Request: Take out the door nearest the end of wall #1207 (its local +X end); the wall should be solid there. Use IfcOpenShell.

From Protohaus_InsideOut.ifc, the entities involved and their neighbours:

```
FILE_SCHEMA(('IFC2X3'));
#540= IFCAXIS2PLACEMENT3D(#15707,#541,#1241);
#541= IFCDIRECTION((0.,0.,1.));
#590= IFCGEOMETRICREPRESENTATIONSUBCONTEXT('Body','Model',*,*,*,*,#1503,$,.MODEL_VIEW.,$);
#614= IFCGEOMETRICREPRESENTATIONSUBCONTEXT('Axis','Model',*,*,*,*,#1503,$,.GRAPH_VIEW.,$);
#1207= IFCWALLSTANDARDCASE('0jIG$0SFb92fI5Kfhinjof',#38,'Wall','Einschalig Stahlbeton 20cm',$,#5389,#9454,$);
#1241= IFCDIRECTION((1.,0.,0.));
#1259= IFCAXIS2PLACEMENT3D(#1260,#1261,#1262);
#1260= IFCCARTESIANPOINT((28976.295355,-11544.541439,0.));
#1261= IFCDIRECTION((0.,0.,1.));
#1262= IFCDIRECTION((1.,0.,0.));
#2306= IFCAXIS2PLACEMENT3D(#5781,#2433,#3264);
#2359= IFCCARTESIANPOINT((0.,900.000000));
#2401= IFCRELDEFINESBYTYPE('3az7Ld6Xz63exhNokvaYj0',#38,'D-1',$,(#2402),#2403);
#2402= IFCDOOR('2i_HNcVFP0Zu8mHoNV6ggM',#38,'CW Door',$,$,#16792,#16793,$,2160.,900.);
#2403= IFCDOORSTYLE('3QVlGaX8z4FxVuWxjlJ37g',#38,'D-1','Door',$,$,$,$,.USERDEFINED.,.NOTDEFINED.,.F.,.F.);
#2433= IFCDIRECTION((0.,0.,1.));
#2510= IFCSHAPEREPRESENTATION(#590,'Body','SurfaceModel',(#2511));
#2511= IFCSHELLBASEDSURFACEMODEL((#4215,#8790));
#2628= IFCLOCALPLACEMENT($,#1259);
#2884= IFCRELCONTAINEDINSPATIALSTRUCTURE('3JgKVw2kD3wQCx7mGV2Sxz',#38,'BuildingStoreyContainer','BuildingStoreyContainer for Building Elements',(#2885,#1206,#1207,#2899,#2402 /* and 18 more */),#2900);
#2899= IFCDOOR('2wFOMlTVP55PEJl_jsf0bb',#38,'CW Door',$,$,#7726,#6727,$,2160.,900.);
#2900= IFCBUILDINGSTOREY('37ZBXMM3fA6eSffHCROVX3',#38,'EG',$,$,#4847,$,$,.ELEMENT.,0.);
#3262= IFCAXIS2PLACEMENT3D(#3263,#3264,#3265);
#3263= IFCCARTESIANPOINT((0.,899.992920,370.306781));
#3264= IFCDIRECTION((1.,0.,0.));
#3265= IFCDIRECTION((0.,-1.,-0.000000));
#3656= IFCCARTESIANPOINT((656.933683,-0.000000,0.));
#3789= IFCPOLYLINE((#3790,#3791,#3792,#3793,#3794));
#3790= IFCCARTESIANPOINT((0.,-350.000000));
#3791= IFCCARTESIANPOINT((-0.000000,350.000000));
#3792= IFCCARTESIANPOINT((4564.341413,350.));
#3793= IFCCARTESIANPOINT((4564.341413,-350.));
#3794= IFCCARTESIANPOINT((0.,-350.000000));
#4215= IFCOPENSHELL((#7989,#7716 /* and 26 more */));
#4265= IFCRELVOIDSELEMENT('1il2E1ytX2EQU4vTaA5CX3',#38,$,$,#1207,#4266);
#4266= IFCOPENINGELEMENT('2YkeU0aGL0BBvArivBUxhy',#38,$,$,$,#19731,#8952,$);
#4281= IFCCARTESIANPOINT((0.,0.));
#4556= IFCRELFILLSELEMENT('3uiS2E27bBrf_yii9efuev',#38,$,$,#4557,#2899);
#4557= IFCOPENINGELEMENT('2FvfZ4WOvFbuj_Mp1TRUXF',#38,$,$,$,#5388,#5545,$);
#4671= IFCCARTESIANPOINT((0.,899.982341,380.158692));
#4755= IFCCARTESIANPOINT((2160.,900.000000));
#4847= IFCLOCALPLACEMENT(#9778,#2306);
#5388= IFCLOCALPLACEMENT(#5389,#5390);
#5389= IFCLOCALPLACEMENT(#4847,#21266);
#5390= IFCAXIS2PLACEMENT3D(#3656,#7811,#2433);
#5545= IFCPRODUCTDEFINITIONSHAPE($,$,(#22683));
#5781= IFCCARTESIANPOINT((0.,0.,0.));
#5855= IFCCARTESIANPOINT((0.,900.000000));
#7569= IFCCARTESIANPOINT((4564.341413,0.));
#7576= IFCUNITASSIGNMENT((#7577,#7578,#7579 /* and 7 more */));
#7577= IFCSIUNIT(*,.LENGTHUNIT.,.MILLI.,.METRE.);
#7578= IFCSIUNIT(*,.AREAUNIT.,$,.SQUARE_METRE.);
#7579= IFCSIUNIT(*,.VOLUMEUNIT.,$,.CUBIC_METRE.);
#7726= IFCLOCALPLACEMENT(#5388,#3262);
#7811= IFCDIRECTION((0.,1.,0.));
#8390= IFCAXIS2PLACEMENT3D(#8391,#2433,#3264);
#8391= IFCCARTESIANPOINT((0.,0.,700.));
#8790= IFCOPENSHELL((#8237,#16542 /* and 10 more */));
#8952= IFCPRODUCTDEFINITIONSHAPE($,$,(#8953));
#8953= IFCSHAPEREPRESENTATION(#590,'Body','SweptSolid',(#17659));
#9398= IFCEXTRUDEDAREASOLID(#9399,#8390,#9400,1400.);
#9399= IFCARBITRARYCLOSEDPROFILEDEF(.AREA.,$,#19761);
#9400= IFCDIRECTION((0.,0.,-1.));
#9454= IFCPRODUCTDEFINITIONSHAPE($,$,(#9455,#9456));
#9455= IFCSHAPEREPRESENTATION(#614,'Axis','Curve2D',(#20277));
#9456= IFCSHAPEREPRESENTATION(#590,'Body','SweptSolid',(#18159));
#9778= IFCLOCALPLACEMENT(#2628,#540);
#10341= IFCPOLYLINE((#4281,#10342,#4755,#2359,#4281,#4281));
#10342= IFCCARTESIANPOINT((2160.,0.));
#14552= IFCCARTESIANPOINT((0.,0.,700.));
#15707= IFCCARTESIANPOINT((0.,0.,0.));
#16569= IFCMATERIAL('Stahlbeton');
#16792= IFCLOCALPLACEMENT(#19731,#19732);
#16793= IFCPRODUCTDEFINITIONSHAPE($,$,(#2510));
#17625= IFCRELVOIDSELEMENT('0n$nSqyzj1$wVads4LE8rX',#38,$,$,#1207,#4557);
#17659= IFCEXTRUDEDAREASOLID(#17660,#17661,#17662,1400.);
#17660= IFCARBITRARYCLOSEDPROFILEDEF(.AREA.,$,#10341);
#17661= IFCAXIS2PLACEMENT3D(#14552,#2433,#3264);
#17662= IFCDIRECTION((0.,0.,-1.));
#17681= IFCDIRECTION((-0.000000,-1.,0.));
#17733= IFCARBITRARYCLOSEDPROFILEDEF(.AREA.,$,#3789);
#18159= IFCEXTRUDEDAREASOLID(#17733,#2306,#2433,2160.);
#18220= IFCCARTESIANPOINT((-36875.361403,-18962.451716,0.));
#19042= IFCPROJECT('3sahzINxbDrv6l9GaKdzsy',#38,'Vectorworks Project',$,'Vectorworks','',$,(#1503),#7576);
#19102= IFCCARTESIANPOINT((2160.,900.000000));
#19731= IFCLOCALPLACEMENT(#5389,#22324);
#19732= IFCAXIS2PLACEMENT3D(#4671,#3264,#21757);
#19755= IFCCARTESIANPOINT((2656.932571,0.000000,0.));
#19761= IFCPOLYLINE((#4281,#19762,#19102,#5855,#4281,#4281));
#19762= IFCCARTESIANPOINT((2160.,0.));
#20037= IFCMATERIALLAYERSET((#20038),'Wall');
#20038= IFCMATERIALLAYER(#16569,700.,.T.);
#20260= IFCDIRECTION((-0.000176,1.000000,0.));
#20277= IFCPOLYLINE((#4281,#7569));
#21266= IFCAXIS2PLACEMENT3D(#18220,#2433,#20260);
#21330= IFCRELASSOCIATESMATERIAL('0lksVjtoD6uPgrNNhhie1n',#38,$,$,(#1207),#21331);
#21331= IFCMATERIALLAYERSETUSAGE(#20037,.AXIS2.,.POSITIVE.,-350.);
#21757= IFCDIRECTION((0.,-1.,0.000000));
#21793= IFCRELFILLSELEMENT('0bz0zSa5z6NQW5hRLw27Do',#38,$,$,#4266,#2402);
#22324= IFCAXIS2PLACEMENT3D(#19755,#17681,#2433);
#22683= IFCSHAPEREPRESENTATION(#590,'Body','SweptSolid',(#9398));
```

```python
import ifcopenshell
import ifcopenshell.api.feature
import ifcopenshell.api.root
import ifcopenshell.geom
import ifcopenshell.util.shape

model = ifcopenshell.open("Protohaus_InsideOut.ifc")
settings = ifcopenshell.geom.settings()


def volume(element):
    """Net volume in cubic metres, openings subtracted."""
    shape = ifcopenshell.geom.create_shape(settings, element)
    return ifcopenshell.util.shape.get_volume(shape.geometry)


door = model.by_guid("2i_HNcVFP0Zu8mHoNV6ggM")
opening = door.FillsVoids[0].RelatingOpeningElement
wall = opening.VoidsElements[0].RelatingBuildingElement
before = volume(wall)

ifcopenshell.api.root.remove_product(model, product=door)
ifcopenshell.api.feature.remove_feature(model, feature=opening)

after = volume(wall)

print(f"wall volume {before:.3f} -> {after:.3f} m3")

model.write("Protohaus_InsideOut_rev.ifc")
```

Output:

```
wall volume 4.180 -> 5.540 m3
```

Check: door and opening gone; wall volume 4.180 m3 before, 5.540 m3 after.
